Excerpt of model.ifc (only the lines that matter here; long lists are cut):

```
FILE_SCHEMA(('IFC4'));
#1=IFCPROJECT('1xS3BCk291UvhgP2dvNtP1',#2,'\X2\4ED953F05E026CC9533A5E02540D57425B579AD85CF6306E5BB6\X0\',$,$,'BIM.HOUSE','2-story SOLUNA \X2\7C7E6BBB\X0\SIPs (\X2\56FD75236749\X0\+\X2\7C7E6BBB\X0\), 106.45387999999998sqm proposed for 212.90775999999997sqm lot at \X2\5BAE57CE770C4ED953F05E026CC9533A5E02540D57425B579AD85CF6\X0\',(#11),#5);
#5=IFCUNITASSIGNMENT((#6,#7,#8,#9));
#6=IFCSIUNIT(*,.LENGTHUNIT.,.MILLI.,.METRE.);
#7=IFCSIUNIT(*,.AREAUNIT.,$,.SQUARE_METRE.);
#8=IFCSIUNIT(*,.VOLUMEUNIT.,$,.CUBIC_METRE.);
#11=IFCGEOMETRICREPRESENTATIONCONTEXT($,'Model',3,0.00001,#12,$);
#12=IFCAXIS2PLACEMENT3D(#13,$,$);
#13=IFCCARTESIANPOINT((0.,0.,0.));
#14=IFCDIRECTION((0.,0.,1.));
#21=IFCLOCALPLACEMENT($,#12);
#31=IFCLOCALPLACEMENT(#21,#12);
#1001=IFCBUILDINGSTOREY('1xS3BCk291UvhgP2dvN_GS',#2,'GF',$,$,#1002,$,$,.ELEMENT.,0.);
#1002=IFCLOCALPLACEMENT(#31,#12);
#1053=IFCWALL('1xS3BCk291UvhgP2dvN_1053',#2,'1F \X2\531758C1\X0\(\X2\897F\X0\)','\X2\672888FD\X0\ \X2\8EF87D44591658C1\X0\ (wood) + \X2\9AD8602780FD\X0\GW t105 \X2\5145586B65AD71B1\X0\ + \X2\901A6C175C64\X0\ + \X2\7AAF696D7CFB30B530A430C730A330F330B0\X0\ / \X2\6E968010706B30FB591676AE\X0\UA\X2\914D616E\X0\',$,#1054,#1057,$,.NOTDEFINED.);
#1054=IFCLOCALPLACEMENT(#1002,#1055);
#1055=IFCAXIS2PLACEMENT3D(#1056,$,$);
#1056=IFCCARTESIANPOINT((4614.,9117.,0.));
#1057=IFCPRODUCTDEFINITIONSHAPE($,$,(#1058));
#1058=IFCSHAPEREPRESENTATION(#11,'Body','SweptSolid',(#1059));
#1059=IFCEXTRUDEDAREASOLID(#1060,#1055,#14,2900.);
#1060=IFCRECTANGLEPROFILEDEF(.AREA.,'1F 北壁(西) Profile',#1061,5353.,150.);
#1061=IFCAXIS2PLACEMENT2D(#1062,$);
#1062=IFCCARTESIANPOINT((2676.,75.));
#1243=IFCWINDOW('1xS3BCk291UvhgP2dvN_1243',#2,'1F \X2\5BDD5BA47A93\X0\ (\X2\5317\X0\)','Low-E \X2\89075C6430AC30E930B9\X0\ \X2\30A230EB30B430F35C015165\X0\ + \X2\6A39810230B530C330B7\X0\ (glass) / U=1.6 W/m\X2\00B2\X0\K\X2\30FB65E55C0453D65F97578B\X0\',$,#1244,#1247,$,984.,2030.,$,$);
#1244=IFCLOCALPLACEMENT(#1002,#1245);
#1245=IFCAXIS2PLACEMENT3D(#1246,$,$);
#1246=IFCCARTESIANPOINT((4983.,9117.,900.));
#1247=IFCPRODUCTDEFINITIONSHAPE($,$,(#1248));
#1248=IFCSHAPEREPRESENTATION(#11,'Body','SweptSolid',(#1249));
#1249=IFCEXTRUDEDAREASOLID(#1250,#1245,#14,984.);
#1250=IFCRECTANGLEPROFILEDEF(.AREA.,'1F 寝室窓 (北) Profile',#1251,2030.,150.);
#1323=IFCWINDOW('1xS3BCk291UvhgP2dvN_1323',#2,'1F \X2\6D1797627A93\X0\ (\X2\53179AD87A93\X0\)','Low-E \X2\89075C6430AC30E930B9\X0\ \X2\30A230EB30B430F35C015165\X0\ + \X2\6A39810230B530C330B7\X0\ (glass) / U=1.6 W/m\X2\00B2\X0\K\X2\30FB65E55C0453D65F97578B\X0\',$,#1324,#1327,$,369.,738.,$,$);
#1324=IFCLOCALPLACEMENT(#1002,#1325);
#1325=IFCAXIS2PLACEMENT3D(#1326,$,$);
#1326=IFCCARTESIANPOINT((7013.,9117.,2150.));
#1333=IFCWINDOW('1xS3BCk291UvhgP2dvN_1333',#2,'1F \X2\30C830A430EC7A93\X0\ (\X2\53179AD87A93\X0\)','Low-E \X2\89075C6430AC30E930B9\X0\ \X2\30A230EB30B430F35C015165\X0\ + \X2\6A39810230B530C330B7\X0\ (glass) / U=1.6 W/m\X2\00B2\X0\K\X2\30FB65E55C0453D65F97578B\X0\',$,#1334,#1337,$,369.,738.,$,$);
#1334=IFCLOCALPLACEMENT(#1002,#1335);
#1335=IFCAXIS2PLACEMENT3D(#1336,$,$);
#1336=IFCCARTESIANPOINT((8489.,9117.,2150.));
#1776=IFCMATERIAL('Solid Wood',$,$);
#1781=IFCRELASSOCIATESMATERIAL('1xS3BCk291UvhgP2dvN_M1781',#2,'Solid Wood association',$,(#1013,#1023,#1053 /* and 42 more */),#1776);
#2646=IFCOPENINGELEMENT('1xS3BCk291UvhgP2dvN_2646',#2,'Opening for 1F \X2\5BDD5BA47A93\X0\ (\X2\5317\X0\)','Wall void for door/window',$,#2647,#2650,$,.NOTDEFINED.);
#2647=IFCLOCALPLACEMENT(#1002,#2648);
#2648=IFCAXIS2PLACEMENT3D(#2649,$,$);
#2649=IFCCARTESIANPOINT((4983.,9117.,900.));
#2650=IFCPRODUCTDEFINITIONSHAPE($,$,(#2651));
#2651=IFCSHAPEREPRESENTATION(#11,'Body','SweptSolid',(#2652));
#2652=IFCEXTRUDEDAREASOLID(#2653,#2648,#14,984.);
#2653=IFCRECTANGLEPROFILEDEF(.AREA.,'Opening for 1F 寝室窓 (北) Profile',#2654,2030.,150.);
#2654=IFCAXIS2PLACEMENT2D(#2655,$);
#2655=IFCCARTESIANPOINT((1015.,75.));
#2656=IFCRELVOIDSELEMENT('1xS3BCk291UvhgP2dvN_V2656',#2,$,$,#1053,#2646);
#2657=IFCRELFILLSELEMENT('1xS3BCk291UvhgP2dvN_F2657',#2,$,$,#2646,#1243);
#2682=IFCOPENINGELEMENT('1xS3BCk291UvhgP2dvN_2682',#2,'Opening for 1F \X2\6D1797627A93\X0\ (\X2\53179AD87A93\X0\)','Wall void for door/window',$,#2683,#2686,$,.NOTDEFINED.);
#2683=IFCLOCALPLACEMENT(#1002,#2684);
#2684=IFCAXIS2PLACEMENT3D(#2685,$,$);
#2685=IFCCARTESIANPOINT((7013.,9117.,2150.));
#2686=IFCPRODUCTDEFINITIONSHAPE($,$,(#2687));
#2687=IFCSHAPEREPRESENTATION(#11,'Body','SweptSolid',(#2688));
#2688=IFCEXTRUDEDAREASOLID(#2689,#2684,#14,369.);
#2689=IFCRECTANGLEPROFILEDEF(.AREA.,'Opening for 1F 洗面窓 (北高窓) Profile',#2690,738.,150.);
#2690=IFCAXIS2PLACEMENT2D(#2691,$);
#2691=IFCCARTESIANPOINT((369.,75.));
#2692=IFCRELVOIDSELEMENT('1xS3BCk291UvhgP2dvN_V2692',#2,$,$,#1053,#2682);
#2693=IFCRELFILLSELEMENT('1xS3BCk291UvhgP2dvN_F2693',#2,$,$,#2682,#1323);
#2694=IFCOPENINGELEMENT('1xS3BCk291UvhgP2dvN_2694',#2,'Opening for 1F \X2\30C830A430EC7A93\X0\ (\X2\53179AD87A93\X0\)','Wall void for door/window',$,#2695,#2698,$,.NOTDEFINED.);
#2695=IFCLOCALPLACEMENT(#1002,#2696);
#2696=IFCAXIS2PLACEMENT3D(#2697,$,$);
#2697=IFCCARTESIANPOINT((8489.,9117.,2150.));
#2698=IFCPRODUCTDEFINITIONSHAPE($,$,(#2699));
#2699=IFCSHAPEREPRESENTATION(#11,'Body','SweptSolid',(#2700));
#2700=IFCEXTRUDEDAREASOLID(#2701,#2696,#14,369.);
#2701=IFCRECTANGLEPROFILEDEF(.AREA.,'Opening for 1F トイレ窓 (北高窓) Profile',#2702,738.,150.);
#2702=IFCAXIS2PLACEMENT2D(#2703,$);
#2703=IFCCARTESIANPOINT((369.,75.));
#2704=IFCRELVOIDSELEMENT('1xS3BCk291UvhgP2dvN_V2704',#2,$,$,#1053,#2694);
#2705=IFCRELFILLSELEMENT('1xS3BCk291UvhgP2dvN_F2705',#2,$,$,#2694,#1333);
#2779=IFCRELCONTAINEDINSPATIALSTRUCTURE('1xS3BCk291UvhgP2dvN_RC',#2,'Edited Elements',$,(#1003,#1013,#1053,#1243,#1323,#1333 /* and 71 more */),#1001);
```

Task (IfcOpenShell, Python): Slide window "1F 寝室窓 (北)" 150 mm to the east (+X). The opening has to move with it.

```python
import ifcopenshell
import ifcopenshell.api.geometry
import ifcopenshell.util.placement

model = ifcopenshell.open("model.ifc")

window = model.by_guid("1xS3BCk291UvhgP2dvN_1243")
opening = window.FillsVoids[0].RelatingOpeningElement
wall = opening.VoidsElements[0].RelatingBuildingElement

wall_matrix = ifcopenshell.util.placement.get_local_placement(wall.ObjectPlacement)
shift = wall_matrix[:3, 0] * 150.0
before = ifcopenshell.util.placement.get_local_placement(window.ObjectPlacement)[:3, 3].copy()

# The window is not placed relative to its opening, so move both.
for product in (opening, window):
    matrix = ifcopenshell.util.placement.get_local_placement(product.ObjectPlacement)
    matrix[:3, 3] += shift
    ifcopenshell.api.geometry.edit_object_placement(model, product=product, matrix=matrix, is_si=False)

after = ifcopenshell.util.placement.get_local_placement(window.ObjectPlacement)[:3, 3]
print("window moved by", (after - before).round(3) + 0.0)

model.write("model_v2.ifc")
```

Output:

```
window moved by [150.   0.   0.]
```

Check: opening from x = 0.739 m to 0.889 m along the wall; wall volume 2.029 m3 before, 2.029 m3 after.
